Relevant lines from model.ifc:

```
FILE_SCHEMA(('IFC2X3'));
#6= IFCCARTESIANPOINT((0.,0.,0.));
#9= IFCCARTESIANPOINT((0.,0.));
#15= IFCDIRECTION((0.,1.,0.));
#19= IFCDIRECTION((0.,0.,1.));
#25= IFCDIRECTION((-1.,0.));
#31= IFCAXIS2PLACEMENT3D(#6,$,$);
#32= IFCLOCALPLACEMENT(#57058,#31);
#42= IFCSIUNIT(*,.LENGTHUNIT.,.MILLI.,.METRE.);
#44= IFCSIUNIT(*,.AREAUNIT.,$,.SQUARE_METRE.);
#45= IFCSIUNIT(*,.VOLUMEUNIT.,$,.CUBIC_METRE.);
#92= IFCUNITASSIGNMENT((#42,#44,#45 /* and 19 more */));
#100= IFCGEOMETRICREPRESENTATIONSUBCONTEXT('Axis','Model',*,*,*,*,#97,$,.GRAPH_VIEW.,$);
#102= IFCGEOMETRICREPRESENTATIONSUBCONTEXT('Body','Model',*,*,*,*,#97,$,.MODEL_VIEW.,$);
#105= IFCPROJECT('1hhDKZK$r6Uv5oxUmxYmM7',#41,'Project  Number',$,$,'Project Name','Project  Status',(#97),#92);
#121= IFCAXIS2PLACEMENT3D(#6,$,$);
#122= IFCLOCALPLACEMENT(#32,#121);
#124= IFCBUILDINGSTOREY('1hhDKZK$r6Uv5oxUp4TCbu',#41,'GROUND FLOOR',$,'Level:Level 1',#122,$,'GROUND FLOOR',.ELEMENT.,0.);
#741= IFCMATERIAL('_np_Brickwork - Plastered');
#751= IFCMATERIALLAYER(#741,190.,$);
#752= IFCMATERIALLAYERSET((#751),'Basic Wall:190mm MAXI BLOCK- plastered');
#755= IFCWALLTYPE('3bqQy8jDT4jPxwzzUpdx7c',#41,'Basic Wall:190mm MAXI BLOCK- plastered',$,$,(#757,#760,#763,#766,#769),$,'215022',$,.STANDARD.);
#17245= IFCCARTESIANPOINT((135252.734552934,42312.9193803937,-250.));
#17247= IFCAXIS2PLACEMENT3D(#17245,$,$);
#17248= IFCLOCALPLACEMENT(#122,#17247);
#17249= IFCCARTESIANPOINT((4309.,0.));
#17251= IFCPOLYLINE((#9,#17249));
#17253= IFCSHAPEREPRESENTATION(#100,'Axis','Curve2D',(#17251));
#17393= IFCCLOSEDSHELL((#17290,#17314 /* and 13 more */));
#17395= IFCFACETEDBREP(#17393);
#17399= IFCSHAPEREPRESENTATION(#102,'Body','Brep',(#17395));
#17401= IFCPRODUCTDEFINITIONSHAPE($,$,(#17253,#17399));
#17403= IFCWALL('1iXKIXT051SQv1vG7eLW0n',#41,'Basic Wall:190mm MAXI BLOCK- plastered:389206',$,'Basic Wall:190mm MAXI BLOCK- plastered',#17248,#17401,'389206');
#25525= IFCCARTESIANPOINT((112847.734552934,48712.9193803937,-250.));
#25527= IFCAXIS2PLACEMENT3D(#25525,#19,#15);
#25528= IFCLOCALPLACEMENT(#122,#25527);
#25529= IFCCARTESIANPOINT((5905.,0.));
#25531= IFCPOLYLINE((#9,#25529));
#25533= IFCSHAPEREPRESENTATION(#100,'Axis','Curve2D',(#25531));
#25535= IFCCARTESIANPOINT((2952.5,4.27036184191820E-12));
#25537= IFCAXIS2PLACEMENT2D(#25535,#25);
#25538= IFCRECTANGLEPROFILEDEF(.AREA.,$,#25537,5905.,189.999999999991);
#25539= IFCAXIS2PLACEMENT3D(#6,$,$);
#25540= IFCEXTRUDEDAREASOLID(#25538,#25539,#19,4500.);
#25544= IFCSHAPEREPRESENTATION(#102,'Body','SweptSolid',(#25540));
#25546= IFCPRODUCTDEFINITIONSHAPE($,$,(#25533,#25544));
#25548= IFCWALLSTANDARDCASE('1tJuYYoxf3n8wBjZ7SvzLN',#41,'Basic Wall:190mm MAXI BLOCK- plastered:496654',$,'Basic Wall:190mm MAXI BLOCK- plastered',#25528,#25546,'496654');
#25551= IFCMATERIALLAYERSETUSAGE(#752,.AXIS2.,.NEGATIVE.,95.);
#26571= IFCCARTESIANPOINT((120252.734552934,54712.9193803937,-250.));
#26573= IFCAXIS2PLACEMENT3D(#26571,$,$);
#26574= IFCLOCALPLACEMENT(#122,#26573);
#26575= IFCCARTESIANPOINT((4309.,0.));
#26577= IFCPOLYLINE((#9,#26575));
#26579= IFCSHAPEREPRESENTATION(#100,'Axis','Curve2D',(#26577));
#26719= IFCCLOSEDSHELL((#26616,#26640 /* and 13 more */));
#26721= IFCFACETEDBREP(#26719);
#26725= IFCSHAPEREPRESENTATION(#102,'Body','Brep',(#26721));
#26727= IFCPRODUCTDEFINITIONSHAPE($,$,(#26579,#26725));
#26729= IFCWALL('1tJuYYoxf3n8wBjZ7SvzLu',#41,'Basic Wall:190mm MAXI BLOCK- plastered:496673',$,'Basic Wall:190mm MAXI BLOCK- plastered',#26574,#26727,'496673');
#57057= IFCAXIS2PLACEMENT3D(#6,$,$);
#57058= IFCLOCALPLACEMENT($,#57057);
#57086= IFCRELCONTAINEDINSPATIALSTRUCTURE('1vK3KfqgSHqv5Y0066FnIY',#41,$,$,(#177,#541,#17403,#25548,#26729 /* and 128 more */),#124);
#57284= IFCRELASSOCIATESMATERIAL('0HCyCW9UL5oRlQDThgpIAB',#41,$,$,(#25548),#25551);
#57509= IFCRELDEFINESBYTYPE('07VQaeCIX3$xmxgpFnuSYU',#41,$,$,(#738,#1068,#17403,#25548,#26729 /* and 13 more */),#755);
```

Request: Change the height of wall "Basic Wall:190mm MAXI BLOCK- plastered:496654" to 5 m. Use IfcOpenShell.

```python
import ifcopenshell
import ifcopenshell.geom
import ifcopenshell.util.representation
import ifcopenshell.util.shape

model = ifcopenshell.open("model.ifc")
settings = ifcopenshell.geom.settings()


def volume(element):
    """Net volume in cubic metres, openings subtracted."""
    shape = ifcopenshell.geom.create_shape(settings, element)
    return ifcopenshell.util.shape.get_volume(shape.geometry)


wall = model.by_guid("1tJuYYoxf3n8wBjZ7SvzLN")
before = volume(wall)

body = ifcopenshell.util.representation.get_representation(wall, "Model", "Body")
solid = body.Items[0]
old_height = solid.Depth
solid.Depth = 5000.0
after = volume(wall)

print(f"height {old_height:g} -> {solid.Depth:g}, volume {before:.3f} -> {after:.3f} m3")

model.write("model_rev.ifc")
```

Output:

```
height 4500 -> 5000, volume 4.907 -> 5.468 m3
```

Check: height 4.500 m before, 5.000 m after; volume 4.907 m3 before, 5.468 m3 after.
